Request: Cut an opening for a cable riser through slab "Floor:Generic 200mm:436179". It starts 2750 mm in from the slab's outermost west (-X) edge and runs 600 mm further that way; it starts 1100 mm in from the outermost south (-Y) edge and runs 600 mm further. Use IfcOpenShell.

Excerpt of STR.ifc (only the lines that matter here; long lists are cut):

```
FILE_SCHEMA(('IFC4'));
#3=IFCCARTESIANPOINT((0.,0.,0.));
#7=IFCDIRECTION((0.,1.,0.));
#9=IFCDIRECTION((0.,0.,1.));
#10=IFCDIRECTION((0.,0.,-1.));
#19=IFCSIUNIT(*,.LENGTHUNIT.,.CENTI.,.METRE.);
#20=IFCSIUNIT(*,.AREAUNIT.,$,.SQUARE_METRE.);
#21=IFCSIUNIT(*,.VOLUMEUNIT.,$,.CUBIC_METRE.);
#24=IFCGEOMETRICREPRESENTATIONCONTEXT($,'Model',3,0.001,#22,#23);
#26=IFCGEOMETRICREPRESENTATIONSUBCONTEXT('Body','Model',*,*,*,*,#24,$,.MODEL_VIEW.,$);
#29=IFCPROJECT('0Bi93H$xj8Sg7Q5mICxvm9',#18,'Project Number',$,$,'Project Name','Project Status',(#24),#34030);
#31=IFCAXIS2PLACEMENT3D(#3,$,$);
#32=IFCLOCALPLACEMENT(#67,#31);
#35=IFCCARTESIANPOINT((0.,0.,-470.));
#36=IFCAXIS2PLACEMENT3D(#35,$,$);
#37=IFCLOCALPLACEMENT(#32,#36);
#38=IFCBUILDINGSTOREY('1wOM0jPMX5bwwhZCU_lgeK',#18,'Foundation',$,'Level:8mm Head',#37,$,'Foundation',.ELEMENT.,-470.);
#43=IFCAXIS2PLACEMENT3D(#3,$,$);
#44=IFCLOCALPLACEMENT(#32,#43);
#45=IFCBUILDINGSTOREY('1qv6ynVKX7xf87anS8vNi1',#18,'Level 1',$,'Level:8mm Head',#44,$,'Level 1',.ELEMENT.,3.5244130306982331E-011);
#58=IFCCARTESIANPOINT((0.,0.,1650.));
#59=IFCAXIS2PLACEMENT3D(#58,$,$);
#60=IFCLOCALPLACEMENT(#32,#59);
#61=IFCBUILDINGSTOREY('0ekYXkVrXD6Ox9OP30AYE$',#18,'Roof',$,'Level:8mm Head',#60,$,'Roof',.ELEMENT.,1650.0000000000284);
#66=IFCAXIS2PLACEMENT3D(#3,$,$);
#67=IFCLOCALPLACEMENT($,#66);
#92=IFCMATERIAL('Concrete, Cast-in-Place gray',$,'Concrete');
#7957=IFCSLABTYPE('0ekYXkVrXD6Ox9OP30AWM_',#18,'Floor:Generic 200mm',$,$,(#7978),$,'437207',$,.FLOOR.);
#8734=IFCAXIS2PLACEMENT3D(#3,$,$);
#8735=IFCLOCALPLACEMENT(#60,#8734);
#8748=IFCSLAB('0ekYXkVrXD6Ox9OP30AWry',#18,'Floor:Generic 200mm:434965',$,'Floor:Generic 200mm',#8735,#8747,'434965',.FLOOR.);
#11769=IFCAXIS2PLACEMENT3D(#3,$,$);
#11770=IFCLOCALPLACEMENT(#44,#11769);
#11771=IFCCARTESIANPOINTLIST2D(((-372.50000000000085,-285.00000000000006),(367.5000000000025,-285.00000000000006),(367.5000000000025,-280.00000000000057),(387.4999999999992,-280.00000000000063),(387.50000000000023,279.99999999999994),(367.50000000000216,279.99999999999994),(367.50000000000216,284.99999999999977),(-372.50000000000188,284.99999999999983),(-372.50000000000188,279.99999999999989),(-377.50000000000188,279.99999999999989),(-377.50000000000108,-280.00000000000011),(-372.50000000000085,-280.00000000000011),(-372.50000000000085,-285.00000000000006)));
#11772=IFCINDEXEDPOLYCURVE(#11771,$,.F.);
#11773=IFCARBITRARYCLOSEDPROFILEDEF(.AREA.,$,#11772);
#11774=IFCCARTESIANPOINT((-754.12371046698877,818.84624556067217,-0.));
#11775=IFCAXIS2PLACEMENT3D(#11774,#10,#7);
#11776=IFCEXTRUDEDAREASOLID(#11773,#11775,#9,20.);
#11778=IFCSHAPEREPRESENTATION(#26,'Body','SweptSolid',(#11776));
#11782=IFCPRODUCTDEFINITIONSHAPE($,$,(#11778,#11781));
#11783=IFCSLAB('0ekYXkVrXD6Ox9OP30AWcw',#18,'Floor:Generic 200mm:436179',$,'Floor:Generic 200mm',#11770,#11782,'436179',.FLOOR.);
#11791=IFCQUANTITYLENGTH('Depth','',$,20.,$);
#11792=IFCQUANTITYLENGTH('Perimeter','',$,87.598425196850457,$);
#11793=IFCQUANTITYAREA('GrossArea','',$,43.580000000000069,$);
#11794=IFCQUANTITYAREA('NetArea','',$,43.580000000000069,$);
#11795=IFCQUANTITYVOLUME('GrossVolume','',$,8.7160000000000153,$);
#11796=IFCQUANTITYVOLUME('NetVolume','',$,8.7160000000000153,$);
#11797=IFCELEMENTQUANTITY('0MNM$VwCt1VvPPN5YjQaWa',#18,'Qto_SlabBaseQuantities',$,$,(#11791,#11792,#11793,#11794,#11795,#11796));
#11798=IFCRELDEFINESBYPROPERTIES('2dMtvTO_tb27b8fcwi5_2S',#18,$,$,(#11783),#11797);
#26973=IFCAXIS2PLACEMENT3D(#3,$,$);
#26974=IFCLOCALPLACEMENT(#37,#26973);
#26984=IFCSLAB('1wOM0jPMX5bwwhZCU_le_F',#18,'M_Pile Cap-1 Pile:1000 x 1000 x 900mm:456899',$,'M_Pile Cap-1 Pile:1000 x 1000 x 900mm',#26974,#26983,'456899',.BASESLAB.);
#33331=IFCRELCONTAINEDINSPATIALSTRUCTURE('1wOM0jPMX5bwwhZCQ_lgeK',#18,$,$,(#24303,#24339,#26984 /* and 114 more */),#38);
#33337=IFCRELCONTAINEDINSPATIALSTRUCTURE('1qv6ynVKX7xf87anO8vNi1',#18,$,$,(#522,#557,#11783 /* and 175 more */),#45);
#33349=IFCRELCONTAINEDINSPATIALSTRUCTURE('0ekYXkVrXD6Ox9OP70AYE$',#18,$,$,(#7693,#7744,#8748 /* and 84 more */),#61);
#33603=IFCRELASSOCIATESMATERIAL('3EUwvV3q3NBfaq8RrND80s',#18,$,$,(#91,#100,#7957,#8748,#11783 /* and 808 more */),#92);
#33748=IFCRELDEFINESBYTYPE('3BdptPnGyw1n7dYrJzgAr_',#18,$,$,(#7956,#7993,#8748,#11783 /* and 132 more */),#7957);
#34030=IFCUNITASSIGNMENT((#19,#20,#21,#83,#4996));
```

```python
import numpy as np
import ifcopenshell
import ifcopenshell.api.feature
import ifcopenshell.api.geometry
import ifcopenshell.api.pset
import ifcopenshell.api.root
import ifcopenshell.geom
import ifcopenshell.util.element
import ifcopenshell.util.placement
import ifcopenshell.util.representation
import ifcopenshell.util.shape
import ifcopenshell.util.unit

model = ifcopenshell.open("STR.ifc")
unit_scale = ifcopenshell.util.unit.calculate_unit_scale(model)
area_scale = ifcopenshell.util.unit.calculate_unit_scale(model, "AREAUNIT")
volume_scale = ifcopenshell.util.unit.calculate_unit_scale(model, "VOLUMEUNIT")
settings = ifcopenshell.geom.settings()


def volume(element):
    """Net volume in cubic metres, openings subtracted."""
    shape = ifcopenshell.geom.create_shape(settings, element)
    return ifcopenshell.util.shape.get_volume(shape.geometry)


slab = model.by_guid("0ekYXkVrXD6Ox9OP30AWcw")
before = volume(slab)

# Extent in the slab's own axes, in metres. The edges named are its -X and -Y sides.
slab_shape = ifcopenshell.geom.create_shape(settings, slab)
vertices = ifcopenshell.util.shape.get_vertices(slab_shape.geometry)
x_min, y_min, bottom = vertices.min(axis=0)
top = vertices[:, 2].max()

opening = ifcopenshell.api.root.create_entity(model, ifc_class="IfcOpeningElement", name="Cable riser opening", predefined_type="OPENING")
context = ifcopenshell.util.representation.get_context(model, "Model", "Body", "MODEL_VIEW")
width, depth = 0.6, 0.6
outline = [(0.0, 0.0), (width, 0.0), (width, depth), (0.0, depth), (0.0, 0.0)]
# Overshoot both faces by 50 mm so the cut is clean.
shape = ifcopenshell.api.geometry.add_slab_representation(
    model, context=context, depth=top - bottom + 0.1, polyline=outline
)
ifcopenshell.api.geometry.assign_representation(model, product=opening, representation=shape)

matrix = ifcopenshell.util.placement.get_local_placement(slab.ObjectPlacement)
matrix[:, 3] = matrix @ np.append(np.array([x_min + 2.75, y_min + 1.1, bottom - 0.05]) / unit_scale, 1.0)
ifcopenshell.api.geometry.edit_object_placement(model, product=opening, matrix=matrix, is_si=False)
ifcopenshell.api.feature.add_feature(model, feature=opening, element=slab)

after = volume(slab)

# Update the slab's stored quantities.
qto = model.by_id(ifcopenshell.util.element.get_pset(slab, "Qto_SlabBaseQuantities", should_inherit=False)["id"])
ifcopenshell.api.pset.edit_qto(model, qto=qto, properties={
    "NetArea": after / (top - bottom) / area_scale,
    "NetVolume": after / volume_scale,
})

print(f"slab volume {before:.3f} -> {after:.3f} m3")

model.write("STR_v2.ifc")
```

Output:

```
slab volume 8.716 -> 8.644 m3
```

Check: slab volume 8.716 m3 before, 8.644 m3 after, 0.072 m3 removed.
